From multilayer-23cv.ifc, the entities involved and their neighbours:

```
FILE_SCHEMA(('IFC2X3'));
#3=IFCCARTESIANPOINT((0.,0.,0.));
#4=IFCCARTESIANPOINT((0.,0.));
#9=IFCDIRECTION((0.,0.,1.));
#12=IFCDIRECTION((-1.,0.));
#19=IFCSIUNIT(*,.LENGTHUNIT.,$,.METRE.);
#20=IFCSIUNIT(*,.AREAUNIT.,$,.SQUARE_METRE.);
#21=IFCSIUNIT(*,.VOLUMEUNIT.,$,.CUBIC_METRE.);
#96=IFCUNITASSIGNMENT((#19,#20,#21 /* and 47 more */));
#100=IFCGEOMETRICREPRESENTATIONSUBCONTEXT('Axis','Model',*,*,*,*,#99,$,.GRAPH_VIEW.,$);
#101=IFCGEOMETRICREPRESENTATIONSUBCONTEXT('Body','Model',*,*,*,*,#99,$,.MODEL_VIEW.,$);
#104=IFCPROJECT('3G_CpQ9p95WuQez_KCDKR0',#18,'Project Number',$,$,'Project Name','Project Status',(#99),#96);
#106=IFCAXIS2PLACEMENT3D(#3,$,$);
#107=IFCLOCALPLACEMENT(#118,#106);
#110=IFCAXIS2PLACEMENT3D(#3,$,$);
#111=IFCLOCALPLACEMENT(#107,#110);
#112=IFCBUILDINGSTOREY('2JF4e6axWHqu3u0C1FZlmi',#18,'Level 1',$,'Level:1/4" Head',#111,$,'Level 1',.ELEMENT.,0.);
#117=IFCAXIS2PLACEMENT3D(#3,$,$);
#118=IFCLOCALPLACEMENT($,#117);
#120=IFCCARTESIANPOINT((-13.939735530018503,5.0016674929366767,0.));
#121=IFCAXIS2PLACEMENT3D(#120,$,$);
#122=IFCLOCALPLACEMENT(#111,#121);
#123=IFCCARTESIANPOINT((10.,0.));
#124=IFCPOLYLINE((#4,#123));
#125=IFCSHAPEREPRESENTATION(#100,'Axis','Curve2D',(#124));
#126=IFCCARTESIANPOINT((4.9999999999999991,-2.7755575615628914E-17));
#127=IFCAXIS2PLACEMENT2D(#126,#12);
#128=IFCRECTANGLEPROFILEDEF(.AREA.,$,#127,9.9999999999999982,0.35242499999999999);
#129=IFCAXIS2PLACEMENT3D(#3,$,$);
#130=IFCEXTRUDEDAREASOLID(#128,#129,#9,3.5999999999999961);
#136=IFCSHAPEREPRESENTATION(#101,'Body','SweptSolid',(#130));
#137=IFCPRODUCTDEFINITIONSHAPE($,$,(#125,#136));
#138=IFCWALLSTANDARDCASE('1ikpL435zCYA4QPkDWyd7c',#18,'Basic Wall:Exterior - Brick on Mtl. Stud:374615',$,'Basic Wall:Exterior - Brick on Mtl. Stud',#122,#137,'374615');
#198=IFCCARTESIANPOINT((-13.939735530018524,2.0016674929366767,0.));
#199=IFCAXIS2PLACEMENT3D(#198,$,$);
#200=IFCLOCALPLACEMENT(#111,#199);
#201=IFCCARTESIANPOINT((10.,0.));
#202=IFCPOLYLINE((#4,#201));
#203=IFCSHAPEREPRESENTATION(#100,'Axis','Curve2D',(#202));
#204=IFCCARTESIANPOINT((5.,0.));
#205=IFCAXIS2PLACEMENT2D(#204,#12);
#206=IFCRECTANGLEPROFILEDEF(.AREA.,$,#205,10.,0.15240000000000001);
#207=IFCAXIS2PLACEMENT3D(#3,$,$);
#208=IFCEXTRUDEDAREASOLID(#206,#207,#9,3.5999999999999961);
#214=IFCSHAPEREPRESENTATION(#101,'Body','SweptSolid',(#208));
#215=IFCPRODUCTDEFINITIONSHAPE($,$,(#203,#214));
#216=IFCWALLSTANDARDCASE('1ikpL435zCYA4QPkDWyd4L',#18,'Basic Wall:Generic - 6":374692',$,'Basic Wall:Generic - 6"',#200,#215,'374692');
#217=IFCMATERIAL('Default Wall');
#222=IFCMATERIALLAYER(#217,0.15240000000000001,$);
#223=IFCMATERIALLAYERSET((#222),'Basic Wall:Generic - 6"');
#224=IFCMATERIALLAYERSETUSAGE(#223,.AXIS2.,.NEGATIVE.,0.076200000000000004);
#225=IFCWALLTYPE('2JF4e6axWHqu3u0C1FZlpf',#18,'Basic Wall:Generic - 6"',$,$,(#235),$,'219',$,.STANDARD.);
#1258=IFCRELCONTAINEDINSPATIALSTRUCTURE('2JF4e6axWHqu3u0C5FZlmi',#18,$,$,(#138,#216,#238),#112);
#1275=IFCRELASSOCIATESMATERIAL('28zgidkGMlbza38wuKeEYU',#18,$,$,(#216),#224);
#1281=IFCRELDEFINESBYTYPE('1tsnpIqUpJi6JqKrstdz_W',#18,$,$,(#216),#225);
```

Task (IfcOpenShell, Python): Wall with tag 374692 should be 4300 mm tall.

```python
import ifcopenshell
import ifcopenshell.geom
import ifcopenshell.util.representation
import ifcopenshell.util.shape
import ifcopenshell.util.unit

model = ifcopenshell.open("multilayer-23cv.ifc")
unit_scale = ifcopenshell.util.unit.calculate_unit_scale(model)
settings = ifcopenshell.geom.settings()


def volume(element):
    """Net volume in cubic metres, openings subtracted."""
    shape = ifcopenshell.geom.create_shape(settings, element)
    return ifcopenshell.util.shape.get_volume(shape.geometry)


wall = model.by_id(216)
before = volume(wall)

body = ifcopenshell.util.representation.get_representation(wall, "Model", "Body")
solid = body.Items[0]
old_height = solid.Depth
solid.Depth = 4.3 / unit_scale
after = volume(wall)

print(f"height {old_height:g} -> {solid.Depth:g}, volume {before:.3f} -> {after:.3f} m3")

model.write("multilayer-23cv-out.ifc")
```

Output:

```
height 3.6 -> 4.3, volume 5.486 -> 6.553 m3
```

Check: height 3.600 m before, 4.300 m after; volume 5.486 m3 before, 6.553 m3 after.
